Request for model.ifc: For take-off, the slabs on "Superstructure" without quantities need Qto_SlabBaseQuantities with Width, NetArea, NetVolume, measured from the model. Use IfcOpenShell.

First a look at what the model holds.

```python
import ifcopenshell
import ifcopenshell.util.element
import ifcopenshell.util.unit

model = ifcopenshell.open("model.ifc")
print(model.schema)
for unit_type in ("LENGTHUNIT", "AREAUNIT", "VOLUMEUNIT"):
    print(unit_type, ifcopenshell.util.unit.calculate_unit_scale(model, unit_type))
storey = next(s for s in model.by_type("IfcBuildingStorey") if s.Name == "Superstructure")
slabs = [e for e in ifcopenshell.util.element.get_decomposition(storey) if e.is_a("IfcSlab")]
for e in sorted(slabs, key=lambda e: e.id()):
    print(e.id(), e.is_a(), e.Name, list(ifcopenshell.util.element.get_psets(e, qtos_only=True)), sep=" | ")
```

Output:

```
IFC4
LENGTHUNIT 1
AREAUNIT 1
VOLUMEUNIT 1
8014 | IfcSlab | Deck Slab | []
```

```python
import ifcopenshell
import ifcopenshell.api.pset
import ifcopenshell.geom
import ifcopenshell.util.element
import ifcopenshell.util.shape
import ifcopenshell.util.unit

model = ifcopenshell.open("model.ifc")
unit_scale = ifcopenshell.util.unit.calculate_unit_scale(model)
area_scale = ifcopenshell.util.unit.calculate_unit_scale(model, "AREAUNIT")
volume_scale = ifcopenshell.util.unit.calculate_unit_scale(model, "VOLUMEUNIT")
settings = ifcopenshell.geom.settings()

storey = next(s for s in model.by_type("IfcBuildingStorey") if s.Name == "Superstructure")
slabs = [e for e in ifcopenshell.util.element.get_decomposition(storey) if e.is_a("IfcSlab")]

for e in sorted(slabs, key=lambda e: e.id()):
    if ifcopenshell.util.element.get_psets(e, qtos_only=True, should_inherit=False):
        continue
    # Geometry comes back in metres, in the element's own axes.
    shape = ifcopenshell.geom.create_shape(settings, e)
    values = {
        "Width": ifcopenshell.util.shape.get_z(shape.geometry) / unit_scale,
        "NetArea": ifcopenshell.util.shape.get_footprint_area(shape.geometry) / area_scale,
        "NetVolume": ifcopenshell.util.shape.get_volume(shape.geometry) / volume_scale,
    }
    qto = ifcopenshell.api.pset.add_qto(model, product=e, name="Qto_SlabBaseQuantities")
    ifcopenshell.api.pset.edit_qto(model, qto=qto, properties=values)
    print(e.id(), {k: round(v, 3) for k, v in values.items()})

model.write("model_v2.ifc")
```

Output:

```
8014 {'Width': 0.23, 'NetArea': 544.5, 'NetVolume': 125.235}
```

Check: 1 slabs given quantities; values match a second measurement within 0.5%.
